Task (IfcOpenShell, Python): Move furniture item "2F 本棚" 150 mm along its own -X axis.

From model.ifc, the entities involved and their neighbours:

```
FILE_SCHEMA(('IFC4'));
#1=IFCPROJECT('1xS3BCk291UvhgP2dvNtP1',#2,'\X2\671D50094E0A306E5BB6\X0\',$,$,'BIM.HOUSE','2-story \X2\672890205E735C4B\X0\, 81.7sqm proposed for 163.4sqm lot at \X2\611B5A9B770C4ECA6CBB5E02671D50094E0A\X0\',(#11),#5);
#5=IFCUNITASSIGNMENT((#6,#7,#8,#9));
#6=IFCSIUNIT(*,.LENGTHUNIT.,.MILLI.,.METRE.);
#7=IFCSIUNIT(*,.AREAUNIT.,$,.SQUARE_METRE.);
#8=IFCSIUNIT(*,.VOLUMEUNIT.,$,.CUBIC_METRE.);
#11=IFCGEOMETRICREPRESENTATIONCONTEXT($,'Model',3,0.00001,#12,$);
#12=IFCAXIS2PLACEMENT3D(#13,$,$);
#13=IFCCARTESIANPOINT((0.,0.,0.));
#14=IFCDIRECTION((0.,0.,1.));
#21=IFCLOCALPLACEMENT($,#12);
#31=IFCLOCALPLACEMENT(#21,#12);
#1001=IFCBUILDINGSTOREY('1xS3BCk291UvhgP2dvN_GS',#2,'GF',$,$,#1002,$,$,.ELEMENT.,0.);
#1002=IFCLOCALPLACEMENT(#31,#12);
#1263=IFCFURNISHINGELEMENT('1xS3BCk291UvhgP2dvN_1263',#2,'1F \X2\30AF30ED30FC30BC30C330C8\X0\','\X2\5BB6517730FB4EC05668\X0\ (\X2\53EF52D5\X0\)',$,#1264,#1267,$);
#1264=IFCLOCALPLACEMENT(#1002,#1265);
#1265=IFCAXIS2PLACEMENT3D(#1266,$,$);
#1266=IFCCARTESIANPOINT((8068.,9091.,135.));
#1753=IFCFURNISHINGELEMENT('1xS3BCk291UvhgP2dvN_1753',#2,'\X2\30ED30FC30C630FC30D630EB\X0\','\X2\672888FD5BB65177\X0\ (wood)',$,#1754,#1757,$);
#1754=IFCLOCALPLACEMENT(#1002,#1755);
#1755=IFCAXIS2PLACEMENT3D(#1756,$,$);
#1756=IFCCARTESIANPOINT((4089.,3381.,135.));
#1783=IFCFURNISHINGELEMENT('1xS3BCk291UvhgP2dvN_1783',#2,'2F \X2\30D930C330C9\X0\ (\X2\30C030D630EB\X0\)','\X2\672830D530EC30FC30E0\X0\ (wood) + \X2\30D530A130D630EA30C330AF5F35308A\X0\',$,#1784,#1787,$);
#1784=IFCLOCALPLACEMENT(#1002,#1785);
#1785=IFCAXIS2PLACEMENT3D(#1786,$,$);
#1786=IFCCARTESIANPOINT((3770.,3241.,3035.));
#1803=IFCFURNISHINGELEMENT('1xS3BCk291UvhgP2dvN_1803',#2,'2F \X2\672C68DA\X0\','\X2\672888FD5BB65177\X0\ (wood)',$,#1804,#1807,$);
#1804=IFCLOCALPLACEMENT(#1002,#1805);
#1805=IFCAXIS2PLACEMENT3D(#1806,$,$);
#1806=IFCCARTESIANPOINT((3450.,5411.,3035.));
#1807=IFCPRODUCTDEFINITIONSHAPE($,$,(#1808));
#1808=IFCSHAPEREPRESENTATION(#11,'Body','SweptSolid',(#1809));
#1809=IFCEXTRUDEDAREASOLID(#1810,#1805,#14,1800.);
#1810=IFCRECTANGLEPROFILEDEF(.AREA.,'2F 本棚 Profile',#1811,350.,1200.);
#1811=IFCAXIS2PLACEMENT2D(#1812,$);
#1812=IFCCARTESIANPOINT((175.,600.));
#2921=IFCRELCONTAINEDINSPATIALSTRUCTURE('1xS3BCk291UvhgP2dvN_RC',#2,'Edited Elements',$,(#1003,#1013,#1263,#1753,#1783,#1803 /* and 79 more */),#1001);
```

```python
import ifcopenshell
import ifcopenshell.api.geometry
import ifcopenshell.util.placement

model = ifcopenshell.open("model.ifc")

item = model.by_id(1803)
matrix = ifcopenshell.util.placement.get_local_placement(item.ObjectPlacement)
matrix[:3, 3] -= matrix[:3, 0] * 150.0
ifcopenshell.api.geometry.edit_object_placement(model, product=item, matrix=matrix, is_si=False)

print(ifcopenshell.util.placement.get_local_placement(item.ObjectPlacement).round(3) + 0.0)

model.write("model_updated.ifc")
```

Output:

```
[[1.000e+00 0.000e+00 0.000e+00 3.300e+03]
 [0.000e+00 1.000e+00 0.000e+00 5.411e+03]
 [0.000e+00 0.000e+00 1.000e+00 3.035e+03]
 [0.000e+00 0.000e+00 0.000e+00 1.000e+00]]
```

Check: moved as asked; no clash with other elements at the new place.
